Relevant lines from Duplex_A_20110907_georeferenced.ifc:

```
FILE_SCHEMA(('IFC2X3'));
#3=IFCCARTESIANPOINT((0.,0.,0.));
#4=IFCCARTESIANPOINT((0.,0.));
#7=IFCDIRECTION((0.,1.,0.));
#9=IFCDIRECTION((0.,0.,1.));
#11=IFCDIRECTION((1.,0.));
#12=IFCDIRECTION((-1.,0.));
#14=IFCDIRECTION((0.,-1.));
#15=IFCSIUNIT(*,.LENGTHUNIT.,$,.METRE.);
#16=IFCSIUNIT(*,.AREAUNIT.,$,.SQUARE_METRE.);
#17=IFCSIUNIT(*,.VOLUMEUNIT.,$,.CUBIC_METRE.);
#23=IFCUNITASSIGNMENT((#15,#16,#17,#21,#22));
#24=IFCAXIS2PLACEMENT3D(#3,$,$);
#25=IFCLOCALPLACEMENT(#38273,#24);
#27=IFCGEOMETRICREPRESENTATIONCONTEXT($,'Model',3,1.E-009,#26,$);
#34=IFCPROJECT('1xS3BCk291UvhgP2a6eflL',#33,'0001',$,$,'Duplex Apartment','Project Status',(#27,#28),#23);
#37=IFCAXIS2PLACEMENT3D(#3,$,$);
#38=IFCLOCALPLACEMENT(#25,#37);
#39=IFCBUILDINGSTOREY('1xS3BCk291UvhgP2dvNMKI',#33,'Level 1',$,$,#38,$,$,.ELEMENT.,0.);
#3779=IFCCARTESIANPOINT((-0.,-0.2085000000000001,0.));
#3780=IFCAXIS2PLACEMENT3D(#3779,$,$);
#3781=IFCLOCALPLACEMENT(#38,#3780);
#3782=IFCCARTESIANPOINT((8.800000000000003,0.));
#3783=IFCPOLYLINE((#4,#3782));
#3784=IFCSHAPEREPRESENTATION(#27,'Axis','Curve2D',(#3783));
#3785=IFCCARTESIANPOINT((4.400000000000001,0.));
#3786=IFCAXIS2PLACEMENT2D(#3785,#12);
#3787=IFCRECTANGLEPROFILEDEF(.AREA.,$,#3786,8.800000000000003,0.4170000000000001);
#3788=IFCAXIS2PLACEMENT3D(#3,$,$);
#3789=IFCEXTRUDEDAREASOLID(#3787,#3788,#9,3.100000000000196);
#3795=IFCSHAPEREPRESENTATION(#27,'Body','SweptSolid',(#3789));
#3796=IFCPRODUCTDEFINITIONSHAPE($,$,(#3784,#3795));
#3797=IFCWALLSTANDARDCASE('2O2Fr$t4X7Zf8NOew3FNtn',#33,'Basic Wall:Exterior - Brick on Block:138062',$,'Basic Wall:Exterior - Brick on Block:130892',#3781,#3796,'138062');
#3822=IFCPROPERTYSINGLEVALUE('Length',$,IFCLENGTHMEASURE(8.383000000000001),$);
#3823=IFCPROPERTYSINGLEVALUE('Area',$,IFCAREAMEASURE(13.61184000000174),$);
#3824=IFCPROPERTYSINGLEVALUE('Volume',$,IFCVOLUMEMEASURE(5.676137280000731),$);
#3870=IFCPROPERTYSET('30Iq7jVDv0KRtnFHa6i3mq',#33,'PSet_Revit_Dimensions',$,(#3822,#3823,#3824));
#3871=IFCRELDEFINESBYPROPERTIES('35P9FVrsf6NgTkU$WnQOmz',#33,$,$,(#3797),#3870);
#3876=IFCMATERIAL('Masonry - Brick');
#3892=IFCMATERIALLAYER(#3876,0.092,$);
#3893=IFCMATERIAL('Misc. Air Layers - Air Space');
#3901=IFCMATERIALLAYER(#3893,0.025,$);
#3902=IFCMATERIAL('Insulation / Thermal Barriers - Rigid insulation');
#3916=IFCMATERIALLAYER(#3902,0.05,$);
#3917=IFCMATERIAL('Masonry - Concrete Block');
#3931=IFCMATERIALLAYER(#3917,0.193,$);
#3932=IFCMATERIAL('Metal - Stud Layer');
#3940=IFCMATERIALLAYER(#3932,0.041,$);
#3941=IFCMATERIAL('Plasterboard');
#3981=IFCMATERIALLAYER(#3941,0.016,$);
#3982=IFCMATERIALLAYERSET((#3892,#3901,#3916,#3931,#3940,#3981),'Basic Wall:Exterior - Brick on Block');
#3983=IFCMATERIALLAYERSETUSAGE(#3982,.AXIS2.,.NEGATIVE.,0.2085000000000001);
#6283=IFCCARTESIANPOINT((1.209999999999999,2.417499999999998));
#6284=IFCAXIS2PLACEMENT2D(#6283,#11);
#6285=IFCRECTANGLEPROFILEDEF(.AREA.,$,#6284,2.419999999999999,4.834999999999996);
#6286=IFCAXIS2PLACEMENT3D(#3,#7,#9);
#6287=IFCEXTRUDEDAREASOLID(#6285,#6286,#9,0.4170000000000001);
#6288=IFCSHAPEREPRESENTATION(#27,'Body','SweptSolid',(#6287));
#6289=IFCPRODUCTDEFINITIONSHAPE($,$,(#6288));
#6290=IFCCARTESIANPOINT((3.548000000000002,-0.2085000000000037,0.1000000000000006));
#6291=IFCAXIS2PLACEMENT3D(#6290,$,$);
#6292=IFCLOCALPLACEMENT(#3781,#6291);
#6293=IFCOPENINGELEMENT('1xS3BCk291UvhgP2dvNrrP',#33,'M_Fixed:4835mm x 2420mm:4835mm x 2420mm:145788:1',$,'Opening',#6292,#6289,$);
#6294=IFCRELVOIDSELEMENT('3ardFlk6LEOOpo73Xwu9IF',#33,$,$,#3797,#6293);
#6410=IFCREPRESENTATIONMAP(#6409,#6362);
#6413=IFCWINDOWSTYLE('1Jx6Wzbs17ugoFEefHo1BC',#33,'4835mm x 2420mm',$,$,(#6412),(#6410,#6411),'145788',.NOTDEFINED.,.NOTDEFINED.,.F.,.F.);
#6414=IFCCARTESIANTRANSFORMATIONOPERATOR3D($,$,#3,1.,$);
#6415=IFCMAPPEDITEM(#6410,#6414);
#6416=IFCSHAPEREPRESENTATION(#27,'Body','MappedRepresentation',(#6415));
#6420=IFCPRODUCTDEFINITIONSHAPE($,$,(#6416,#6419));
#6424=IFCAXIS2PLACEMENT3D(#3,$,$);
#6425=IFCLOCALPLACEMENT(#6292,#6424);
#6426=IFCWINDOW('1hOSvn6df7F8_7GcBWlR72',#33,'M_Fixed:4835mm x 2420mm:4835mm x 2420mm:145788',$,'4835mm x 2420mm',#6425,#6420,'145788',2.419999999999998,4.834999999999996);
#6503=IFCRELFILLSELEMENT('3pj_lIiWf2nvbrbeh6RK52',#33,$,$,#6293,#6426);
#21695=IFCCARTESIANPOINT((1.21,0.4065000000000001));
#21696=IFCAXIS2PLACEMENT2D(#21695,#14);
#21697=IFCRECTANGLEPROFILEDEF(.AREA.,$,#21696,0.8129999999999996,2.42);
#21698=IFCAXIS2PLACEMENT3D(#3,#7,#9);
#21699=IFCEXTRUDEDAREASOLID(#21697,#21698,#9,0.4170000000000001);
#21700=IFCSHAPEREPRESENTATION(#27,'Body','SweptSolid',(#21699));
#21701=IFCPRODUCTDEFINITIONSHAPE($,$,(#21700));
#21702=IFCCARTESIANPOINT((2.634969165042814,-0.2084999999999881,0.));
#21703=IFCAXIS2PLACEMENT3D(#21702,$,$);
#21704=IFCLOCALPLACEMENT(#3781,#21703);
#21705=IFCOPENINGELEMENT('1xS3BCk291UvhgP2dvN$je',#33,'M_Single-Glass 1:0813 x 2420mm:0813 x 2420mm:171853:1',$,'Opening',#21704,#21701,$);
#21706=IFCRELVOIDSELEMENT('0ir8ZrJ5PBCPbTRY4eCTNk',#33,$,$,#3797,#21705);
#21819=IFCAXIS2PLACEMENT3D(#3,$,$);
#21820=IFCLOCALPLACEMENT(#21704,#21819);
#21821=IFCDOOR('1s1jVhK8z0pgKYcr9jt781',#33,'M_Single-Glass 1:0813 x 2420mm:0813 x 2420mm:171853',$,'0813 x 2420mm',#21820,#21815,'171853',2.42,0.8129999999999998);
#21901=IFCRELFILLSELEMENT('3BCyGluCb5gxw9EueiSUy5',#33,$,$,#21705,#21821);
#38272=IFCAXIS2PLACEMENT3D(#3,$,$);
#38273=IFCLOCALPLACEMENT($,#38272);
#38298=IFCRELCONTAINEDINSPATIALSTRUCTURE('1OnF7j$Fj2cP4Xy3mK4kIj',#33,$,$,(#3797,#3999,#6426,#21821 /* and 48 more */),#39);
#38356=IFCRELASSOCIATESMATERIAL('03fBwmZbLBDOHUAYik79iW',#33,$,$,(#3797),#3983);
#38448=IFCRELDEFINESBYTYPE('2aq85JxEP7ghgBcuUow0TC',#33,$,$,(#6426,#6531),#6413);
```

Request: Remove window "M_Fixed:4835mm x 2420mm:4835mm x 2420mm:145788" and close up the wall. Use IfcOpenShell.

```python
import ifcopenshell
import ifcopenshell.api.feature
import ifcopenshell.api.pset
import ifcopenshell.api.root
import ifcopenshell.geom
import ifcopenshell.util.element
import ifcopenshell.util.shape
import ifcopenshell.util.unit

model = ifcopenshell.open("Duplex_A_20110907_georeferenced.ifc")
area_scale = ifcopenshell.util.unit.calculate_unit_scale(model, "AREAUNIT")
volume_scale = ifcopenshell.util.unit.calculate_unit_scale(model, "VOLUMEUNIT")
settings = ifcopenshell.geom.settings()


def volume(element):
    """Net volume in cubic metres, openings subtracted."""
    shape = ifcopenshell.geom.create_shape(settings, element)
    return ifcopenshell.util.shape.get_volume(shape.geometry)


window = model.by_id(6426)
opening = window.FillsVoids[0].RelatingOpeningElement
wall = opening.VoidsElements[0].RelatingBuildingElement
before = volume(wall)

ifcopenshell.api.root.remove_product(model, product=window)
ifcopenshell.api.feature.remove_feature(model, feature=opening)

after = volume(wall)
thickness = 0.417  # wall thickness in metres

# Update the wall's stored quantities.
pset = model.by_id(ifcopenshell.util.element.get_pset(wall, "PSet_Revit_Dimensions", should_inherit=False)["id"])
ifcopenshell.api.pset.edit_pset(model, pset=pset, properties={
    "Area": model.create_entity("IfcAreaMeasure", after / thickness / area_scale),
    "Volume": model.create_entity("IfcVolumeMeasure", after / volume_scale),
})

print(f"wall volume {before:.3f} -> {after:.3f} m3")

model.write("Duplex_A_20110907_georeferenced_rev.ifc")
```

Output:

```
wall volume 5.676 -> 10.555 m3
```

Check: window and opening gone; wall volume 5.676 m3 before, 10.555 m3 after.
